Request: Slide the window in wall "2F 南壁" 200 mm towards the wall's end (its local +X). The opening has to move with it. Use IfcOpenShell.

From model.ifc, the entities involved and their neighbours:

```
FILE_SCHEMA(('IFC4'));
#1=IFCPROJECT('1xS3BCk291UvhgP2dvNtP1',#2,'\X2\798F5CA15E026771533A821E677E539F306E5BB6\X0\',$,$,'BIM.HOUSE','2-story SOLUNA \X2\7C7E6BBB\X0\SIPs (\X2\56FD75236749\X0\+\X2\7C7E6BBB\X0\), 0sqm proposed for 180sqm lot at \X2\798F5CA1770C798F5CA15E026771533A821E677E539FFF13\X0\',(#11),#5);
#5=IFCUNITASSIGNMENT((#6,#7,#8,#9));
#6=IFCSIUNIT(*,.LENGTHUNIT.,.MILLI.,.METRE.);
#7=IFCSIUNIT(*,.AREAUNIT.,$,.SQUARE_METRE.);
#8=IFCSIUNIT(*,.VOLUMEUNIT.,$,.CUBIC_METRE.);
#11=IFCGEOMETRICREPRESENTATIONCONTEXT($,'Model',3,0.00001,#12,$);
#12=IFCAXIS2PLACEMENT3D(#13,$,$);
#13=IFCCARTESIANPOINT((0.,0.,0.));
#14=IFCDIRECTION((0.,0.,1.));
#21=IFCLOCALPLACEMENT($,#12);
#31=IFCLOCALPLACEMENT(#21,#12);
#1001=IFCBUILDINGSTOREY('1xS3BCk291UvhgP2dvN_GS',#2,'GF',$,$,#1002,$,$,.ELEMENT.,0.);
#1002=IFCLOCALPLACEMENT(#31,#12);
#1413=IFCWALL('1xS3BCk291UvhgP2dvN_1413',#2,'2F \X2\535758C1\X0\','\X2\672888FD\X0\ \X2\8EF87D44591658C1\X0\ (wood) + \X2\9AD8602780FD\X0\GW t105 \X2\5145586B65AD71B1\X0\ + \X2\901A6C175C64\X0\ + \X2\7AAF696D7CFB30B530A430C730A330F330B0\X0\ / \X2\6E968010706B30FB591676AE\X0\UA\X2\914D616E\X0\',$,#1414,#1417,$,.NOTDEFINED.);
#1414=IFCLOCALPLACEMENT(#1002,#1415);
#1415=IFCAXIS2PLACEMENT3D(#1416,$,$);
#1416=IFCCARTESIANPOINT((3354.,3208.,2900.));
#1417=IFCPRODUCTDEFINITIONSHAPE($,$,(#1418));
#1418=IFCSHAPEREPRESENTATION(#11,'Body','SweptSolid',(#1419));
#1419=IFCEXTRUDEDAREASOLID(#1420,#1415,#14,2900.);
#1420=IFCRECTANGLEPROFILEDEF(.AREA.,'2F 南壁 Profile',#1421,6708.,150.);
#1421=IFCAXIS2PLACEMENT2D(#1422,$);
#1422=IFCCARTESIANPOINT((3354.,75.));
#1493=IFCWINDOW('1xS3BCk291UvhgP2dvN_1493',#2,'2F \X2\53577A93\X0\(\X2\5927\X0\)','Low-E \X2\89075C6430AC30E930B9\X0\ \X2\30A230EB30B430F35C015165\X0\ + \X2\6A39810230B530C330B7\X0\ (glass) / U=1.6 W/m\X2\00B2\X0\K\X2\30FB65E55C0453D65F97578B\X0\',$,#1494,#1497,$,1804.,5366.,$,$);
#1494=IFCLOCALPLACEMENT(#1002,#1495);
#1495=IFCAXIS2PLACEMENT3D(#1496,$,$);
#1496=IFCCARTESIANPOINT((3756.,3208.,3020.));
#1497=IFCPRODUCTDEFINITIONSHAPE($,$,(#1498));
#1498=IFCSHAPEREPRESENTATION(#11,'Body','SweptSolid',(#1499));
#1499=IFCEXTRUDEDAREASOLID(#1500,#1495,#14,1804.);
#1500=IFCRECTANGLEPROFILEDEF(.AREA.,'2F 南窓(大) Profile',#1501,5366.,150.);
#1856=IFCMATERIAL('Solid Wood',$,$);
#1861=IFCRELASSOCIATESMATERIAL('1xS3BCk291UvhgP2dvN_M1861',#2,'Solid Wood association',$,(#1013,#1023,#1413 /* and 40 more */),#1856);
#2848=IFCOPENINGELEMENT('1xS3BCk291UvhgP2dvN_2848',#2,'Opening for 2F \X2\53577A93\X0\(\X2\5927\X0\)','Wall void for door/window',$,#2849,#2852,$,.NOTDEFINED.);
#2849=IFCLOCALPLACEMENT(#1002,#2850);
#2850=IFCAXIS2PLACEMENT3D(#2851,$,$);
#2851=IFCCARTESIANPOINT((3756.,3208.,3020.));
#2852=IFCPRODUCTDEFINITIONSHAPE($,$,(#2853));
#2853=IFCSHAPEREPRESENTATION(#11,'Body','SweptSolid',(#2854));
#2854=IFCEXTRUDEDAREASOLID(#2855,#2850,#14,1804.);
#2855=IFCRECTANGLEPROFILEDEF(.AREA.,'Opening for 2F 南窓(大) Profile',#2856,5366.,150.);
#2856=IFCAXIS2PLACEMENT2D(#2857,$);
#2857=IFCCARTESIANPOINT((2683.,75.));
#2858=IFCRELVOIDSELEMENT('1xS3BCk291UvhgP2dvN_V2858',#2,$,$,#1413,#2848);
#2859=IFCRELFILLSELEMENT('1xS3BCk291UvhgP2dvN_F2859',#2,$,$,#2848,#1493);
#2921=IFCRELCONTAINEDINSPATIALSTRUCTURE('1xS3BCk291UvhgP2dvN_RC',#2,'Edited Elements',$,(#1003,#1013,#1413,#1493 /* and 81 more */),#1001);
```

```python
import ifcopenshell
import ifcopenshell.api.geometry
import ifcopenshell.util.placement

model = ifcopenshell.open("model.ifc")

window = model.by_guid("1xS3BCk291UvhgP2dvN_1493")
opening = window.FillsVoids[0].RelatingOpeningElement
wall = opening.VoidsElements[0].RelatingBuildingElement

wall_matrix = ifcopenshell.util.placement.get_local_placement(wall.ObjectPlacement)
shift = wall_matrix[:3, 0] * 200.0
before = ifcopenshell.util.placement.get_local_placement(window.ObjectPlacement)[:3, 3].copy()

# The window is not placed relative to its opening, so move both.
for product in (opening, window):
    matrix = ifcopenshell.util.placement.get_local_placement(product.ObjectPlacement)
    matrix[:3, 3] += shift
    ifcopenshell.api.geometry.edit_object_placement(model, product=product, matrix=matrix, is_si=False)

after = ifcopenshell.util.placement.get_local_placement(window.ObjectPlacement)[:3, 3]
print("window moved by", (after - before).round(3) + 0.0)

model.write("model_rev.ifc")
```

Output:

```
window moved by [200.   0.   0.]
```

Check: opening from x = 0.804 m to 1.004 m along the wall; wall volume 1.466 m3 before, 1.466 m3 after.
